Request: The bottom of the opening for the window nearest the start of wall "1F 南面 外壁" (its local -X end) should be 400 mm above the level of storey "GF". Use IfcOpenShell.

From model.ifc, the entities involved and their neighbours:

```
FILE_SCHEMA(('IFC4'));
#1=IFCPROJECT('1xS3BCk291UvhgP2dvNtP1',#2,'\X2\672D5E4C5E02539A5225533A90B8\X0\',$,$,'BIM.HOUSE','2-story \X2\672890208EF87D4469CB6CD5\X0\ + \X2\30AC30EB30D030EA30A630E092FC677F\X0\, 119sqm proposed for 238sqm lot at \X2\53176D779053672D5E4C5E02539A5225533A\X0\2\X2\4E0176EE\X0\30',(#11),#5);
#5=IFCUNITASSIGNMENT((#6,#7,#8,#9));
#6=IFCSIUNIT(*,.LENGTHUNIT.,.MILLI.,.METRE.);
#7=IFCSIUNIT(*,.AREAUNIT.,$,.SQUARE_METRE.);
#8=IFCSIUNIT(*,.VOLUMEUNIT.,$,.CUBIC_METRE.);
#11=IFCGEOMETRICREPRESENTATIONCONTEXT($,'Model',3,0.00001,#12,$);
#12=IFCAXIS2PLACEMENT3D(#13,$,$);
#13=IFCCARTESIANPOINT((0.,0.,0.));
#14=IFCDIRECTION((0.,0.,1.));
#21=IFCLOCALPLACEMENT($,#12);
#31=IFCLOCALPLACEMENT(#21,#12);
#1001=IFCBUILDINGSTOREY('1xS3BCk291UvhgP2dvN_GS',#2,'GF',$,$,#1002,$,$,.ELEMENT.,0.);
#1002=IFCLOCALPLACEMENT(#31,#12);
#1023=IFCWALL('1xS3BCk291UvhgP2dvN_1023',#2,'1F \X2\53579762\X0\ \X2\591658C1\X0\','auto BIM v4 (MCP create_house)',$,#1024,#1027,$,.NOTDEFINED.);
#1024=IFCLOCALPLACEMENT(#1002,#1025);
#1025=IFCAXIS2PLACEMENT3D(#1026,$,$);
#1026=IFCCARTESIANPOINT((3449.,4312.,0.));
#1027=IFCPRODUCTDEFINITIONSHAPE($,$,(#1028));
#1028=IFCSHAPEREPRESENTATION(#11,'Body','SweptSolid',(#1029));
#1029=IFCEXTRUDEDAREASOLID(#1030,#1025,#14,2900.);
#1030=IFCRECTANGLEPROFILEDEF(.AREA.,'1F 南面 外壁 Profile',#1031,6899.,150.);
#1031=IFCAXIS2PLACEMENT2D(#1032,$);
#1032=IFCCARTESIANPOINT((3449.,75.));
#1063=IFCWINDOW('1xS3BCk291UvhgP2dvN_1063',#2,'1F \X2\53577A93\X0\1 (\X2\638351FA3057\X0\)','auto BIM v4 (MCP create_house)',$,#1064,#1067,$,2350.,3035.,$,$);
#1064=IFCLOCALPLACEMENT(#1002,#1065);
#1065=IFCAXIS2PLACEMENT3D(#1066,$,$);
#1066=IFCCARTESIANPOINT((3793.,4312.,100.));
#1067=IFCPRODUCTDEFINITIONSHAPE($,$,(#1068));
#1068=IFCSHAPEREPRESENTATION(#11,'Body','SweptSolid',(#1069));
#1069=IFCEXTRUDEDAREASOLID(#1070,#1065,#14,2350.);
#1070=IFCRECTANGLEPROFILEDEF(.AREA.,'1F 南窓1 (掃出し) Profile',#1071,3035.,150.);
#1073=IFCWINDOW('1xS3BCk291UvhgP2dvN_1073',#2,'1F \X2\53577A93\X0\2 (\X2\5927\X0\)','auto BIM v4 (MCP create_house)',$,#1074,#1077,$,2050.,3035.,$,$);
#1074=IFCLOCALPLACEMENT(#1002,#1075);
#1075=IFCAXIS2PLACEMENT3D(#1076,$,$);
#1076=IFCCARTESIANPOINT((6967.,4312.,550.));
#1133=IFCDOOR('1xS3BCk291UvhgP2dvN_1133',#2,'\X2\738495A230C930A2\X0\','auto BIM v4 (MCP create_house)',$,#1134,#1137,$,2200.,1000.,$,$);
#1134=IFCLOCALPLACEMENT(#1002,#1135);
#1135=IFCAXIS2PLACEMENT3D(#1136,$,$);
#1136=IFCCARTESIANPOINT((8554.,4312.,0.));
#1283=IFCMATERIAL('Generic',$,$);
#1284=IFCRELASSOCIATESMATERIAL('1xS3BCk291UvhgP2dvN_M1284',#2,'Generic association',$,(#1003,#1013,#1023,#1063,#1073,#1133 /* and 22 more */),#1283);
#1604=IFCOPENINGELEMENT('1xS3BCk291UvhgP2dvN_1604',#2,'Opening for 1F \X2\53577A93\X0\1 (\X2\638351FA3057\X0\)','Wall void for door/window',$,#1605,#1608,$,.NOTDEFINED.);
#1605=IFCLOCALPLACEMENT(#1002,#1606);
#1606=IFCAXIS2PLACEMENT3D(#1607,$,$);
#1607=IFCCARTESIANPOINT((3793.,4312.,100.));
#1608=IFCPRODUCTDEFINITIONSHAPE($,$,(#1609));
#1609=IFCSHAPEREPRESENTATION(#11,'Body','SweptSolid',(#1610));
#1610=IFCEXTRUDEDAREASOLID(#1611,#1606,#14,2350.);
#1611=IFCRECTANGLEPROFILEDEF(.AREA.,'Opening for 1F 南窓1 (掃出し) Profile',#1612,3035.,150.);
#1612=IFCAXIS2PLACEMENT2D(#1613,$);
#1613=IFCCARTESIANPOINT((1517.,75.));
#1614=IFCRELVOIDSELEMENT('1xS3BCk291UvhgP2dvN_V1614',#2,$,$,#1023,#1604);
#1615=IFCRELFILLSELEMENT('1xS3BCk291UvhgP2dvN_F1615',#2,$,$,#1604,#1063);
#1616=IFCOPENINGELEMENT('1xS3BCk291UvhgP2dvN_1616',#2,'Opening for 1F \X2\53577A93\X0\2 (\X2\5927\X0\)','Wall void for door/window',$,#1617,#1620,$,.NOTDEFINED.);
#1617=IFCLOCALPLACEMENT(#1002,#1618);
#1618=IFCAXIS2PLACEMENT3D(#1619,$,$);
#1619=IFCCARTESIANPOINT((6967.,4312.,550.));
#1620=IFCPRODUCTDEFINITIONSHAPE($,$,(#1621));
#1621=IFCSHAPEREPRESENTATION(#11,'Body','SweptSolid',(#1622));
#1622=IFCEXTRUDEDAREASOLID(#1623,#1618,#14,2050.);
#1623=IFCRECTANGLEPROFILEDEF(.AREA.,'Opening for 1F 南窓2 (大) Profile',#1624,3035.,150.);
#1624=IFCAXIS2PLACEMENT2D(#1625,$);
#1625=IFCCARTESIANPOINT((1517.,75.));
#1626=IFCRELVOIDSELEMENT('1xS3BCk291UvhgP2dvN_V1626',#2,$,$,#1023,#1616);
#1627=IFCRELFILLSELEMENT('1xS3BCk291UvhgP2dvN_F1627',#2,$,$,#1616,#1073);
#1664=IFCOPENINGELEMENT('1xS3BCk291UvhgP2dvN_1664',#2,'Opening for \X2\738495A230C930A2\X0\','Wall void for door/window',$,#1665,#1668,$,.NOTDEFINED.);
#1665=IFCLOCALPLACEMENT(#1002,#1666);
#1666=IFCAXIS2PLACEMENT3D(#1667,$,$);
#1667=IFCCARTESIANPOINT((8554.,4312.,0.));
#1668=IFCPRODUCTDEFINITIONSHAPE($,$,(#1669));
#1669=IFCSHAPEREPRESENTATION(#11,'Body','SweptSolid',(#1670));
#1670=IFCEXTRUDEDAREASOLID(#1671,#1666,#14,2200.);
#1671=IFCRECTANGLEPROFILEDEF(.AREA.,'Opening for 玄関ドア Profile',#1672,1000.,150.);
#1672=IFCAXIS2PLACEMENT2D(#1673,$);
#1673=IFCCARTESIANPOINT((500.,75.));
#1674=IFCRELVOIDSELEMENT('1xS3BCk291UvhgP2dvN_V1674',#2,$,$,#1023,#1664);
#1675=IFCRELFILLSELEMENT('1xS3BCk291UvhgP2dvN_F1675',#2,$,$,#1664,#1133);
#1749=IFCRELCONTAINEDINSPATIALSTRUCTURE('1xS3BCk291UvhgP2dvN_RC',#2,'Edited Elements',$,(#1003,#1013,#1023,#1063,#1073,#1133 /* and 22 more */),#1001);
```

```python
import numpy as np
import ifcopenshell
import ifcopenshell.api.geometry
import ifcopenshell.geom
import ifcopenshell.util.element
import ifcopenshell.util.placement
import ifcopenshell.util.shape
import ifcopenshell.util.unit

model = ifcopenshell.open("model.ifc")
unit_scale = ifcopenshell.util.unit.calculate_unit_scale(model)

window = model.by_guid("1xS3BCk291UvhgP2dvN_1063")
opening = window.FillsVoids[0].RelatingOpeningElement
storey = ifcopenshell.util.element.get_container(window, ifc_class="IfcBuildingStorey")
level = ifcopenshell.util.placement.get_local_placement(storey.ObjectPlacement)[2, 3]

# The opening's origin need not be at the sill, so measure its lowest point.
shape = ifcopenshell.geom.create_shape(ifcopenshell.geom.settings(), opening)
bottom = ifcopenshell.util.shape.get_shape_bottom_elevation(shape, shape.geometry) / unit_scale
dz = level + 0.4 / unit_scale - bottom

shift = np.array([0.0, 0.0, dz])
# The window is not placed relative to its opening, so move both.
for product in (opening, window):
    matrix = ifcopenshell.util.placement.get_local_placement(product.ObjectPlacement)
    matrix[:3, 3] += shift
    ifcopenshell.api.geometry.edit_object_placement(model, product=product, matrix=matrix, is_si=False)

print(f"moved by {dz * unit_scale:+.3f} m")

model.write("model_rev.ifc")
```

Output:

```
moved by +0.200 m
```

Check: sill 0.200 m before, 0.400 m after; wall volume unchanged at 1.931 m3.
